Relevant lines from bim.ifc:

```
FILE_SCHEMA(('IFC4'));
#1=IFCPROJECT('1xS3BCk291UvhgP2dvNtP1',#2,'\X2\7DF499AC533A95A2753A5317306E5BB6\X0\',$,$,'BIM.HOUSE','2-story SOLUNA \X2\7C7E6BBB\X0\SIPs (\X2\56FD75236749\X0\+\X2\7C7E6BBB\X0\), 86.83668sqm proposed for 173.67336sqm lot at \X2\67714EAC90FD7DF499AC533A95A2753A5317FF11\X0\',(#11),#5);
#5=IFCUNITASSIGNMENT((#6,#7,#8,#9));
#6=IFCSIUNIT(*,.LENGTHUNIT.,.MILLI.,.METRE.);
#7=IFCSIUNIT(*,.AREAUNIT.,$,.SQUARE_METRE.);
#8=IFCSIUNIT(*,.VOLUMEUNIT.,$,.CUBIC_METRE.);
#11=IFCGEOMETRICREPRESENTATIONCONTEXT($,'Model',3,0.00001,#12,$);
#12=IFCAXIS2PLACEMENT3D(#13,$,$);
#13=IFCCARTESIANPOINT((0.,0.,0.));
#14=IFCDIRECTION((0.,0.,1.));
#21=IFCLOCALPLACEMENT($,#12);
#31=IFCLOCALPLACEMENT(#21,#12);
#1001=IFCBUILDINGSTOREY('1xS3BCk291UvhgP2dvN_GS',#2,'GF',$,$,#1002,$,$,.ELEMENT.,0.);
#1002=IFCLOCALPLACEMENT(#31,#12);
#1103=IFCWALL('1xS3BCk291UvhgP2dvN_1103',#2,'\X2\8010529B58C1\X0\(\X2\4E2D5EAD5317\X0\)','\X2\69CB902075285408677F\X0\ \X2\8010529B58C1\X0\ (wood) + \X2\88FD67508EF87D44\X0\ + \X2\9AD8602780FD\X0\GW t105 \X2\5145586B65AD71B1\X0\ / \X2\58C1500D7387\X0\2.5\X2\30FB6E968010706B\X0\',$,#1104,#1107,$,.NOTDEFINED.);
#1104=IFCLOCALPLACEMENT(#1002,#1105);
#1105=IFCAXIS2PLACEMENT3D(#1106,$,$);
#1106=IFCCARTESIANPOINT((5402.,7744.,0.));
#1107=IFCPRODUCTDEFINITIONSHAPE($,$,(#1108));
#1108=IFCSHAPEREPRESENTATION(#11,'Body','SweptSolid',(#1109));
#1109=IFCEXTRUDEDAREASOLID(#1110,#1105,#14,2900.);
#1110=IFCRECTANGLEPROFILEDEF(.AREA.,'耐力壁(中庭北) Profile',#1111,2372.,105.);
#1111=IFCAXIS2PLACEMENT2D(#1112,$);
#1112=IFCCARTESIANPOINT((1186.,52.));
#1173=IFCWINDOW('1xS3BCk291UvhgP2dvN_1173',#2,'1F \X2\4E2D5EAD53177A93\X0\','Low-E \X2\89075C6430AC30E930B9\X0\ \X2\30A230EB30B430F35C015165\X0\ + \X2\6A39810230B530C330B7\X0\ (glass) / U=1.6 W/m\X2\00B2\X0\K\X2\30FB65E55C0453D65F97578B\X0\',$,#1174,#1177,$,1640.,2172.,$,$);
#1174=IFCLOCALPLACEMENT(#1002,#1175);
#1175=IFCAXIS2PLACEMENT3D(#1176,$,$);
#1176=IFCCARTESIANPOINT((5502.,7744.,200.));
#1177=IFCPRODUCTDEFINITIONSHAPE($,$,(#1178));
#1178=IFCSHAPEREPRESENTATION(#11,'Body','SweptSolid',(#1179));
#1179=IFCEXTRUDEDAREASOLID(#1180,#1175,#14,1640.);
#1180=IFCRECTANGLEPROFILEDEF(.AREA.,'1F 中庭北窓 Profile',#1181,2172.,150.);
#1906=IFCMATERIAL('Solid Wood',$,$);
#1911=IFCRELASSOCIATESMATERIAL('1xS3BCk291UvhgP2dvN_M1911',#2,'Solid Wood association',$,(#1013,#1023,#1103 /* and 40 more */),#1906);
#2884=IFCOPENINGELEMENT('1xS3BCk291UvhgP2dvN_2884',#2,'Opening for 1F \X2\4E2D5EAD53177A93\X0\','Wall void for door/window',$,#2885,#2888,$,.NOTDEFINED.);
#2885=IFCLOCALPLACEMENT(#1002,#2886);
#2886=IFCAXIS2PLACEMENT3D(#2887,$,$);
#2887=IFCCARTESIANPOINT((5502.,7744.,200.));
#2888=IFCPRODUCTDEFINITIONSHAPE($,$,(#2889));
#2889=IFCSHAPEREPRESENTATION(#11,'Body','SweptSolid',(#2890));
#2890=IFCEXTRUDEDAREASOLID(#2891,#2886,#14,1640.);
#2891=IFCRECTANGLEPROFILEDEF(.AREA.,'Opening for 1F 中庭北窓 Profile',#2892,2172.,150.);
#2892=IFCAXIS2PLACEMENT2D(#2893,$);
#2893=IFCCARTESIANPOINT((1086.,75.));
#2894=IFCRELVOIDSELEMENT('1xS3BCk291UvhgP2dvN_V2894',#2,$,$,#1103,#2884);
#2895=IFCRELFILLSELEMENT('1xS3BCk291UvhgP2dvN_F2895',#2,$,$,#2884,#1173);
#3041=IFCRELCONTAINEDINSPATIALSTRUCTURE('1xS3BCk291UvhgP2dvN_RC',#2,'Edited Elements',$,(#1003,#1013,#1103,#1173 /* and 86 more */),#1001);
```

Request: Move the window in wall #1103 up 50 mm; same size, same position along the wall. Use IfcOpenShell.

```python
import numpy as np
import ifcopenshell
import ifcopenshell.api.geometry
import ifcopenshell.util.placement
import ifcopenshell.util.unit

model = ifcopenshell.open("bim.ifc")
unit_scale = ifcopenshell.util.unit.calculate_unit_scale(model)

window = model.by_guid("1xS3BCk291UvhgP2dvN_1173")
opening = window.FillsVoids[0].RelatingOpeningElement
dz = 50.0

shift = np.array([0.0, 0.0, dz])
# The window is not placed relative to its opening, so move both.
for product in (opening, window):
    matrix = ifcopenshell.util.placement.get_local_placement(product.ObjectPlacement)
    matrix[:3, 3] += shift
    ifcopenshell.api.geometry.edit_object_placement(model, product=product, matrix=matrix, is_si=False)

print(f"moved by {dz * unit_scale:+.3f} m")

model.write("bim_edited.ifc")
```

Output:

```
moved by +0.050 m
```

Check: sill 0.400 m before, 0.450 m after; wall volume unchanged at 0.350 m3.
